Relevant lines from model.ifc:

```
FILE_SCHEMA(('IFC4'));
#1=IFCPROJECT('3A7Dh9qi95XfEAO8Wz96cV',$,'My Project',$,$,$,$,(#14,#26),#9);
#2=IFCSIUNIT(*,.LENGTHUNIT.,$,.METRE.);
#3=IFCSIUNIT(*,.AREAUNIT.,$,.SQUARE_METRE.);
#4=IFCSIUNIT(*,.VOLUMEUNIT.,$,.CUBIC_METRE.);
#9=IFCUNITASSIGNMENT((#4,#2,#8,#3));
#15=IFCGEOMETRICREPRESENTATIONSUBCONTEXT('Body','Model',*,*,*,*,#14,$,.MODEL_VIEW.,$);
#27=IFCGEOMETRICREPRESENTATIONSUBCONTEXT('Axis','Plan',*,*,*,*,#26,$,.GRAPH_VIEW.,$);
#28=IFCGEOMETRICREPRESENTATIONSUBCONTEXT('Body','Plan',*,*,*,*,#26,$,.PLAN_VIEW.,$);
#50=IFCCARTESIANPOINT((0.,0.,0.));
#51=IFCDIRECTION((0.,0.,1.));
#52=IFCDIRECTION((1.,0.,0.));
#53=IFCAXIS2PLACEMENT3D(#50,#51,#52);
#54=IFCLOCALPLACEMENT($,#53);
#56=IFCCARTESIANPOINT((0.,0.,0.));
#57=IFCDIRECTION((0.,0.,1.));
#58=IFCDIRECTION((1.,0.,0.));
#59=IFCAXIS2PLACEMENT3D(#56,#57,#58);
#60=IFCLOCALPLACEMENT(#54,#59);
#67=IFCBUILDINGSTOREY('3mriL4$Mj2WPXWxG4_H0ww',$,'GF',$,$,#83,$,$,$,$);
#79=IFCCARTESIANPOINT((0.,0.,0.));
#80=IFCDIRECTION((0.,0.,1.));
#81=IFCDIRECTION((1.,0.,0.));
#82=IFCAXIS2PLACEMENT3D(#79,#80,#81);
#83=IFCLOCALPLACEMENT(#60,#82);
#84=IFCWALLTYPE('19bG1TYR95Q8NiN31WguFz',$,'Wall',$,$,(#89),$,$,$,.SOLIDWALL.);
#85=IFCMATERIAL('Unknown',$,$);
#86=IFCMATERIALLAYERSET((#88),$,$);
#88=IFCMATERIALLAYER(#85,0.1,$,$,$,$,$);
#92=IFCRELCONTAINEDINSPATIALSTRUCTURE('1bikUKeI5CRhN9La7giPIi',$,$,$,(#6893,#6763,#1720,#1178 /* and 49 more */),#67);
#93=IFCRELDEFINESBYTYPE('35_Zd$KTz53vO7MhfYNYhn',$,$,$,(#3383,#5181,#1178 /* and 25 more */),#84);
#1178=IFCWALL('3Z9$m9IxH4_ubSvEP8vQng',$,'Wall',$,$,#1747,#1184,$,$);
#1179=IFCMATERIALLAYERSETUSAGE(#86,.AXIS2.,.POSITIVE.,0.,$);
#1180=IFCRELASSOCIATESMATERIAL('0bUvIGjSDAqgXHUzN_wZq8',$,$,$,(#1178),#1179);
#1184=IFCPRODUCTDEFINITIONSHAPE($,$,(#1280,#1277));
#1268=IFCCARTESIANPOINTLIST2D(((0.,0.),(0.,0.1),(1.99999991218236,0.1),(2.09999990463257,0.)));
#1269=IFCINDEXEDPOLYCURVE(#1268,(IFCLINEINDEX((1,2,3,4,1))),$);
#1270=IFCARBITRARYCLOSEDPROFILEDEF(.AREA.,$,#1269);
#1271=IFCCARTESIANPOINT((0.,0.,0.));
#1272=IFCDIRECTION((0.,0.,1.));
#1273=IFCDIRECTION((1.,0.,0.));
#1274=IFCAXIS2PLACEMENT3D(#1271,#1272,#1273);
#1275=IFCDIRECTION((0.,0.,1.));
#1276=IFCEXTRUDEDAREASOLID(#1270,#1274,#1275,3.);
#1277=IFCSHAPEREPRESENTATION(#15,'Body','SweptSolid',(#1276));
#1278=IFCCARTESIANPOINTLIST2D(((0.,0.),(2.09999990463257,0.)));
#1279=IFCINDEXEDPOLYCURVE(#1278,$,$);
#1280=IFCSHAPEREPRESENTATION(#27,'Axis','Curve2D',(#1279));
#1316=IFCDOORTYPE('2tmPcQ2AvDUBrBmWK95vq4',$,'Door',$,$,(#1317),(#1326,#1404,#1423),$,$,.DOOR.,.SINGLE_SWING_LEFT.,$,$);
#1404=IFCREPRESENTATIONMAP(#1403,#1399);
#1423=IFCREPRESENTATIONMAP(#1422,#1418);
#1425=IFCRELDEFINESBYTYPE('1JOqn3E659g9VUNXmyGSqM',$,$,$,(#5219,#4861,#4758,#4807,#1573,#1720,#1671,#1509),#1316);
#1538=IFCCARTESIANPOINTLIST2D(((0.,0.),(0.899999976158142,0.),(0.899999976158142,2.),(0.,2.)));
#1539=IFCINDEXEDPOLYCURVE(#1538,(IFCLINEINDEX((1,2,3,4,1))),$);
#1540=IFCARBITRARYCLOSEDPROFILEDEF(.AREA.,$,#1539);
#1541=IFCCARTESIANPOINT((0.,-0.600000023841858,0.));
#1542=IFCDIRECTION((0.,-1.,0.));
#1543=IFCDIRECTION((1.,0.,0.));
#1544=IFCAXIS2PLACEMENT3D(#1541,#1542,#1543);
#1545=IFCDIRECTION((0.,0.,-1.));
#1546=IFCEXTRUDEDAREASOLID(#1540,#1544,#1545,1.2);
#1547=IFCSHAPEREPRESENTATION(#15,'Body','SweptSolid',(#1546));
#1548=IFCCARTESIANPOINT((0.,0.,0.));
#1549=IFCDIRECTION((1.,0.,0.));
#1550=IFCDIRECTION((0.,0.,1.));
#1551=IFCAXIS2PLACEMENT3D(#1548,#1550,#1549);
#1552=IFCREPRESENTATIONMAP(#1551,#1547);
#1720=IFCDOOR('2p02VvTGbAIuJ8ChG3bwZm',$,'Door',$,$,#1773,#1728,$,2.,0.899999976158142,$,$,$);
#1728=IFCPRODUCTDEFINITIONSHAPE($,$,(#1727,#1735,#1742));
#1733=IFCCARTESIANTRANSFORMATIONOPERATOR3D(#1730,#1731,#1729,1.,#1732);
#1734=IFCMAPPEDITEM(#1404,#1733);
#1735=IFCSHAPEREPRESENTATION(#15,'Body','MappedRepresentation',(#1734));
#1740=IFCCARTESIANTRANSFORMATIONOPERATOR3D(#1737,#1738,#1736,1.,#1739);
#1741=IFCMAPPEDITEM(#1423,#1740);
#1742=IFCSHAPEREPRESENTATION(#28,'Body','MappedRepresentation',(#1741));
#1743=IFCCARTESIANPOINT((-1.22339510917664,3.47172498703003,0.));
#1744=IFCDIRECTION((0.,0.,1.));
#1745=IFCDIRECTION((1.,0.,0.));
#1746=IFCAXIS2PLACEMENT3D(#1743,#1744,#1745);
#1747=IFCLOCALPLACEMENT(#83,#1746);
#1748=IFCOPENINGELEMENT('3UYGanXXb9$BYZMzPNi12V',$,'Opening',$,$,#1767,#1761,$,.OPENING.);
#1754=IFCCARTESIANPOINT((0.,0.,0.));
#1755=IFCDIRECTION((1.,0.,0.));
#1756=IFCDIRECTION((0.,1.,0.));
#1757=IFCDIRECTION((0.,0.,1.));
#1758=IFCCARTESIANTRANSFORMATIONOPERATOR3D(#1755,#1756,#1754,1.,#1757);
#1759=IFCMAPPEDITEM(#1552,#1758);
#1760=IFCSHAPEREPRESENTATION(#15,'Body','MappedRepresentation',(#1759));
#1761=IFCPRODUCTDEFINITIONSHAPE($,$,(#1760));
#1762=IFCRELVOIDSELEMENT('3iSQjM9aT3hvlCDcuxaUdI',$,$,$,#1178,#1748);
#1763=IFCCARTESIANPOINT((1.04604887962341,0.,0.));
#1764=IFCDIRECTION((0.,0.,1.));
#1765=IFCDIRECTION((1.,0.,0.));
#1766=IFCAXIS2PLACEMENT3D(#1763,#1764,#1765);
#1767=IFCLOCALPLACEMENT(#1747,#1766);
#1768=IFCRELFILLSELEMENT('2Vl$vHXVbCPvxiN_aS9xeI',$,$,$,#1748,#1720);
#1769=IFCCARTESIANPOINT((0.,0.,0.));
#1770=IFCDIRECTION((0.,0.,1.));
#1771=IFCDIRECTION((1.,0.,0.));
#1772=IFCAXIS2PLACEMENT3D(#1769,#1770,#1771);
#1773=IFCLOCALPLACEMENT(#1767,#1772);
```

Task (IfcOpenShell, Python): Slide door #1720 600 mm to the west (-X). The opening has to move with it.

```python
import ifcopenshell
import ifcopenshell.api.geometry
import ifcopenshell.util.placement

model = ifcopenshell.open("model.ifc")

door = model.by_id(1720)
opening = door.FillsVoids[0].RelatingOpeningElement
wall = opening.VoidsElements[0].RelatingBuildingElement

wall_matrix = ifcopenshell.util.placement.get_local_placement(wall.ObjectPlacement)
shift = wall_matrix[:3, 0] * -0.6
before = ifcopenshell.util.placement.get_local_placement(door.ObjectPlacement)[:3, 3].copy()

# The door is placed relative to its opening, so it follows when the opening moves.
matrix = ifcopenshell.util.placement.get_local_placement(opening.ObjectPlacement)
matrix[:3, 3] += shift
ifcopenshell.api.geometry.edit_object_placement(
    model, product=opening, matrix=matrix, is_si=False, should_transform_children=True
)

after = ifcopenshell.util.placement.get_local_placement(door.ObjectPlacement)[:3, 3]
print("door moved by", (after - before).round(3) + 0.0)

model.write("model-out.ifc")
```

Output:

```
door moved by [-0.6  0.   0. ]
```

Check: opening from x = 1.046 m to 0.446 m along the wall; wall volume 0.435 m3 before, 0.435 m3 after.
